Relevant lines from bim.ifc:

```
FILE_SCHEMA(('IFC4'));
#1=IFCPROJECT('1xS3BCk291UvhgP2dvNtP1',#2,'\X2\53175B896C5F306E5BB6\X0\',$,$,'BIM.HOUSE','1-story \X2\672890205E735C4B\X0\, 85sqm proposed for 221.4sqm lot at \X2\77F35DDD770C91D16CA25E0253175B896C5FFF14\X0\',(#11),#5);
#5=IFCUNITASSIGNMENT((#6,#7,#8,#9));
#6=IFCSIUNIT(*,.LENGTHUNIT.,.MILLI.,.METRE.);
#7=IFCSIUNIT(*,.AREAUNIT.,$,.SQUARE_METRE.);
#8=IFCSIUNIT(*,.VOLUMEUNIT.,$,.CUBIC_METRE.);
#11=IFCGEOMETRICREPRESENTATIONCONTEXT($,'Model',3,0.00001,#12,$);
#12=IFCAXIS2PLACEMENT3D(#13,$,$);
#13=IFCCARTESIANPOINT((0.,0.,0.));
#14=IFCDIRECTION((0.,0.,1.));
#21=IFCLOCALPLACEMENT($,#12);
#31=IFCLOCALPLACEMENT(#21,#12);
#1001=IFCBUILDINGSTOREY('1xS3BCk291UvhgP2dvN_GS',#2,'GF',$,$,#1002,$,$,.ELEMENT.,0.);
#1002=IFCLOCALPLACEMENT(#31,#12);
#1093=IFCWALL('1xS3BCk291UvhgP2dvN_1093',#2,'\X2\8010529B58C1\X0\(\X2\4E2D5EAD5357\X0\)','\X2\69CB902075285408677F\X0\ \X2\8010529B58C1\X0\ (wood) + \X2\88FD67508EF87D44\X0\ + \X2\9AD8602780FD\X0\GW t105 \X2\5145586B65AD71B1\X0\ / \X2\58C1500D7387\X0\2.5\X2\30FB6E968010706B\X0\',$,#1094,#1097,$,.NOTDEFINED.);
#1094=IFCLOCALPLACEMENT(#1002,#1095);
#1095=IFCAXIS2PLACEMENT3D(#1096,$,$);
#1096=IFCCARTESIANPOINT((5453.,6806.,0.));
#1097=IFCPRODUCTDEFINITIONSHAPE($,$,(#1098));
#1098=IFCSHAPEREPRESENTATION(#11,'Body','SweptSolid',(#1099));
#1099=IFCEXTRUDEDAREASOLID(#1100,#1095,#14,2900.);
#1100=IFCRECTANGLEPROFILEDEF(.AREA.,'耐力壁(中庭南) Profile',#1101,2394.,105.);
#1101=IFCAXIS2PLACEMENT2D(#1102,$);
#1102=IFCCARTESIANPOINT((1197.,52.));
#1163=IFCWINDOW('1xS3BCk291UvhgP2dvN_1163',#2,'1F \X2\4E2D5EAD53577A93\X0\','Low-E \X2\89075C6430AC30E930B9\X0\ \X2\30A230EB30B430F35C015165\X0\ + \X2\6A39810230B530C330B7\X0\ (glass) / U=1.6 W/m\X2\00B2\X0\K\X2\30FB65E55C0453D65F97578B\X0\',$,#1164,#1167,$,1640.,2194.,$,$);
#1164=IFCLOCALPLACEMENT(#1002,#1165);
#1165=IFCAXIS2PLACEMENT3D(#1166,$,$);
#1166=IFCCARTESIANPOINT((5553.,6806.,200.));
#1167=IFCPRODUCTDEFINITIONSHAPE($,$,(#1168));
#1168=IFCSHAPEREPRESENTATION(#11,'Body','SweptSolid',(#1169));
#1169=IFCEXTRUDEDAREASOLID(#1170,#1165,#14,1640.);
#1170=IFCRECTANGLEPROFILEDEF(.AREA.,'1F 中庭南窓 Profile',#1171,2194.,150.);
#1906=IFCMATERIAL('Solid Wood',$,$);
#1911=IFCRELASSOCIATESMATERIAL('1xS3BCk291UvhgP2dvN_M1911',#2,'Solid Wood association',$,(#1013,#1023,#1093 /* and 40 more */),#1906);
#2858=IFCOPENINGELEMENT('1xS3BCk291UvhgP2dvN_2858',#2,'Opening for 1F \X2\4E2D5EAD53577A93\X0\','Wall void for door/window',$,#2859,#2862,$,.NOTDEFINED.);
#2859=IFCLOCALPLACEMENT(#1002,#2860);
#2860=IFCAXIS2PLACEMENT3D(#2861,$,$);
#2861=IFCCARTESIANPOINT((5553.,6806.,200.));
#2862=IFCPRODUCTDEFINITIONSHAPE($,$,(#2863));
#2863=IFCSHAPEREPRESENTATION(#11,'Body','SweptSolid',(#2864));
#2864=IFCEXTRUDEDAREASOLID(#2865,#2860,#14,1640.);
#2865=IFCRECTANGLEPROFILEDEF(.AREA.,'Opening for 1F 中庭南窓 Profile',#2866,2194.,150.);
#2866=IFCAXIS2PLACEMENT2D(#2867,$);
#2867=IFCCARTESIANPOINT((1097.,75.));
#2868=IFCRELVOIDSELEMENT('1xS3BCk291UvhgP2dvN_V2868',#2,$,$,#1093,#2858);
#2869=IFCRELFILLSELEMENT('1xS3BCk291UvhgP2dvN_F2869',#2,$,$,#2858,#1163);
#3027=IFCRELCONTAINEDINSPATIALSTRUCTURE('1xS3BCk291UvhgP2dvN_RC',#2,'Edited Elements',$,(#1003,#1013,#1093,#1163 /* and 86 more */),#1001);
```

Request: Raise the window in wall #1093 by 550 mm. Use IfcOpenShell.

```python
import numpy as np
import ifcopenshell
import ifcopenshell.api.geometry
import ifcopenshell.util.placement
import ifcopenshell.util.unit

model = ifcopenshell.open("bim.ifc")
unit_scale = ifcopenshell.util.unit.calculate_unit_scale(model)

window = model.by_guid("1xS3BCk291UvhgP2dvN_1163")
opening = window.FillsVoids[0].RelatingOpeningElement
dz = 0.55 / unit_scale

shift = np.array([0.0, 0.0, dz])
# The window is not placed relative to its opening, so move both.
for product in (opening, window):
    matrix = ifcopenshell.util.placement.get_local_placement(product.ObjectPlacement)
    matrix[:3, 3] += shift
    ifcopenshell.api.geometry.edit_object_placement(model, product=product, matrix=matrix, is_si=False)

print(f"moved by {dz * unit_scale:+.3f} m")

model.write("bim_rev.ifc")
```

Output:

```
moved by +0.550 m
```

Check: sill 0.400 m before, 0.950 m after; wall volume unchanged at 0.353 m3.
